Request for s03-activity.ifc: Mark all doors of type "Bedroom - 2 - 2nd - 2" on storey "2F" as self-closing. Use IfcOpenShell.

First a look at what the model holds.

```python
import ifcopenshell
import ifcopenshell.util.element

model = ifcopenshell.open("s03-activity.ifc")
print(model.schema)
storey = next(s for s in model.by_type("IfcBuildingStorey") if s.Name == "2F")
doors = [e for e in ifcopenshell.util.element.get_decomposition(storey) if e.is_a("IfcDoor")]
seen = {}
for e in doors:
    element_type = ifcopenshell.util.element.get_type(e)
    key = (element_type.Name if element_type != e and element_type else None, ifcopenshell.util.element.get_pset(e, "Pset_DoorCommon", "SelfClosing"))
    seen[key] = seen.get(key, 0) + 1
for (name, value), count in sorted(seen.items(), key=str):
    print(count, "x", name, "|", value)
```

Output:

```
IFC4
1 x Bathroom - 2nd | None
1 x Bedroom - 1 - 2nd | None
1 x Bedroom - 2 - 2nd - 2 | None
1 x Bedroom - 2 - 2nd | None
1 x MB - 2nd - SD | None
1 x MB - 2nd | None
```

```python
import ifcopenshell
import ifcopenshell.api.pset
import ifcopenshell.util.element

model = ifcopenshell.open("s03-activity.ifc")

storey = next(s for s in model.by_type("IfcBuildingStorey") if s.Name == "2F")
doors = [e for e in ifcopenshell.util.element.get_decomposition(storey) if e.is_a("IfcDoor")]

count = 0
for e in doors:
    element_type = ifcopenshell.util.element.get_type(e)
    if element_type in (None, e) or element_type.Name != "Bedroom - 2 - 2nd - 2":
        continue
    # add_pset returns the element's existing set when there is one.
    pset = ifcopenshell.api.pset.add_pset(model, product=e, name="Pset_DoorCommon")
    ifcopenshell.api.pset.edit_pset(model, pset=pset, properties={"SelfClosing": True})
    count += 1

print(count, "doors updated")

model.write("s03-activity_v2.ifc")
```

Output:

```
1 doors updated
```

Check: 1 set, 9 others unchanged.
